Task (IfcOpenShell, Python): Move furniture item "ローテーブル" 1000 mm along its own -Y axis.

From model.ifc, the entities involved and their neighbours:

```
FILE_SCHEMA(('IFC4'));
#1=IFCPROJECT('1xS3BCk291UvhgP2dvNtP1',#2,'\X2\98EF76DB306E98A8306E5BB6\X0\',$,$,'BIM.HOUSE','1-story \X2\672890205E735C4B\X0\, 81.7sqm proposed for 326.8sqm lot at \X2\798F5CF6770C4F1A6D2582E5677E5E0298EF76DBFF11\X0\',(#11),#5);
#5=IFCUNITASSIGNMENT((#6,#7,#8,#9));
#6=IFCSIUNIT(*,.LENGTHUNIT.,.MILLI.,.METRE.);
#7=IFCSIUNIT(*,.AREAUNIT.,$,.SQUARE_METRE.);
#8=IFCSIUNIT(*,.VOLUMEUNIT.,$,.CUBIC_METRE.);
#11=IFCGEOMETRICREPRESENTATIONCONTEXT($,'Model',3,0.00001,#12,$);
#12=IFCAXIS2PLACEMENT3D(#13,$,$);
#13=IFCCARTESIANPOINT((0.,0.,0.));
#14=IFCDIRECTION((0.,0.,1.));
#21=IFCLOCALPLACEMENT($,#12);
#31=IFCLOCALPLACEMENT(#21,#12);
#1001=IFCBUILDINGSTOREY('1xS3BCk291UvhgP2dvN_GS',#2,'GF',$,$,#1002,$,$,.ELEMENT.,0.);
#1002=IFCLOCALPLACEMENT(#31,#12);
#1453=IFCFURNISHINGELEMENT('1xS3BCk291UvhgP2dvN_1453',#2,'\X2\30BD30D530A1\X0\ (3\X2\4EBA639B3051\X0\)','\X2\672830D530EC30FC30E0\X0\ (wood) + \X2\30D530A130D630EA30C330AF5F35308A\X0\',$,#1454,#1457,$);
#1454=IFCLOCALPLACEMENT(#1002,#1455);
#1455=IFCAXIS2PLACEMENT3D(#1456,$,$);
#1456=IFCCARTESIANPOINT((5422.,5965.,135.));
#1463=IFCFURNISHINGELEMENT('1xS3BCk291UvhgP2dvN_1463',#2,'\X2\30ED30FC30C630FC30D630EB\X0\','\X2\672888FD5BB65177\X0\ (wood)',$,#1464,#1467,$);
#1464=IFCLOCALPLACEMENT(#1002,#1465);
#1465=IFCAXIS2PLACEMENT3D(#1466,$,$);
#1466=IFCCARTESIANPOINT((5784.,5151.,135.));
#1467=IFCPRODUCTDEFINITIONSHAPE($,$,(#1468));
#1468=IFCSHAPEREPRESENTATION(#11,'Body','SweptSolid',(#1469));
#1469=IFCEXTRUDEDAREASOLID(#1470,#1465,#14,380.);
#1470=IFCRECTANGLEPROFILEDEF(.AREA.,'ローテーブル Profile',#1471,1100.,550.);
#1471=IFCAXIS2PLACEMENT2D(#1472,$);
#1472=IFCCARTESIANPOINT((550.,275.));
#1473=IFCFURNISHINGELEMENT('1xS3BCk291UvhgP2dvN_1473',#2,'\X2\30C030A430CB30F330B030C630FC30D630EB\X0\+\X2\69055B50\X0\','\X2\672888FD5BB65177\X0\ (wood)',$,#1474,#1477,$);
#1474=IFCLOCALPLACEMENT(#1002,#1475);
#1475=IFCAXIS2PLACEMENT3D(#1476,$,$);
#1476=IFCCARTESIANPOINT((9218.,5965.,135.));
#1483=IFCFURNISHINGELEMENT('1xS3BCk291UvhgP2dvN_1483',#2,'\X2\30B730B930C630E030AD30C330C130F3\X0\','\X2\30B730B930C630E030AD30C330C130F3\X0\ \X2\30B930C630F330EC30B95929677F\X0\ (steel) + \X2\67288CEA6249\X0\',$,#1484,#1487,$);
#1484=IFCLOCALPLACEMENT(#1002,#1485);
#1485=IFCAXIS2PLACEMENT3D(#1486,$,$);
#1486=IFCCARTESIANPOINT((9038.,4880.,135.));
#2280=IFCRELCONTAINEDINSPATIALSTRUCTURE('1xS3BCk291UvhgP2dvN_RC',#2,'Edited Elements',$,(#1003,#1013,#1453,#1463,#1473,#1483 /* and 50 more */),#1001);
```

```python
import ifcopenshell
import ifcopenshell.api.geometry
import ifcopenshell.util.placement
import ifcopenshell.util.unit

model = ifcopenshell.open("model.ifc")
unit_scale = ifcopenshell.util.unit.calculate_unit_scale(model)

item = model.by_guid("1xS3BCk291UvhgP2dvN_1463")
matrix = ifcopenshell.util.placement.get_local_placement(item.ObjectPlacement)
matrix[:3, 3] -= matrix[:3, 1] * 1 / unit_scale
ifcopenshell.api.geometry.edit_object_placement(model, product=item, matrix=matrix, is_si=False)

print(ifcopenshell.util.placement.get_local_placement(item.ObjectPlacement).round(3) + 0.0)

model.write("model-out.ifc")
```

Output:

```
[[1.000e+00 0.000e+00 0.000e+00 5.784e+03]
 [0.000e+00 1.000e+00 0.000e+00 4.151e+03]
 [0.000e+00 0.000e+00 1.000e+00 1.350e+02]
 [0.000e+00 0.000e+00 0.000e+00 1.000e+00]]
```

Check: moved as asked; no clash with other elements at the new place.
